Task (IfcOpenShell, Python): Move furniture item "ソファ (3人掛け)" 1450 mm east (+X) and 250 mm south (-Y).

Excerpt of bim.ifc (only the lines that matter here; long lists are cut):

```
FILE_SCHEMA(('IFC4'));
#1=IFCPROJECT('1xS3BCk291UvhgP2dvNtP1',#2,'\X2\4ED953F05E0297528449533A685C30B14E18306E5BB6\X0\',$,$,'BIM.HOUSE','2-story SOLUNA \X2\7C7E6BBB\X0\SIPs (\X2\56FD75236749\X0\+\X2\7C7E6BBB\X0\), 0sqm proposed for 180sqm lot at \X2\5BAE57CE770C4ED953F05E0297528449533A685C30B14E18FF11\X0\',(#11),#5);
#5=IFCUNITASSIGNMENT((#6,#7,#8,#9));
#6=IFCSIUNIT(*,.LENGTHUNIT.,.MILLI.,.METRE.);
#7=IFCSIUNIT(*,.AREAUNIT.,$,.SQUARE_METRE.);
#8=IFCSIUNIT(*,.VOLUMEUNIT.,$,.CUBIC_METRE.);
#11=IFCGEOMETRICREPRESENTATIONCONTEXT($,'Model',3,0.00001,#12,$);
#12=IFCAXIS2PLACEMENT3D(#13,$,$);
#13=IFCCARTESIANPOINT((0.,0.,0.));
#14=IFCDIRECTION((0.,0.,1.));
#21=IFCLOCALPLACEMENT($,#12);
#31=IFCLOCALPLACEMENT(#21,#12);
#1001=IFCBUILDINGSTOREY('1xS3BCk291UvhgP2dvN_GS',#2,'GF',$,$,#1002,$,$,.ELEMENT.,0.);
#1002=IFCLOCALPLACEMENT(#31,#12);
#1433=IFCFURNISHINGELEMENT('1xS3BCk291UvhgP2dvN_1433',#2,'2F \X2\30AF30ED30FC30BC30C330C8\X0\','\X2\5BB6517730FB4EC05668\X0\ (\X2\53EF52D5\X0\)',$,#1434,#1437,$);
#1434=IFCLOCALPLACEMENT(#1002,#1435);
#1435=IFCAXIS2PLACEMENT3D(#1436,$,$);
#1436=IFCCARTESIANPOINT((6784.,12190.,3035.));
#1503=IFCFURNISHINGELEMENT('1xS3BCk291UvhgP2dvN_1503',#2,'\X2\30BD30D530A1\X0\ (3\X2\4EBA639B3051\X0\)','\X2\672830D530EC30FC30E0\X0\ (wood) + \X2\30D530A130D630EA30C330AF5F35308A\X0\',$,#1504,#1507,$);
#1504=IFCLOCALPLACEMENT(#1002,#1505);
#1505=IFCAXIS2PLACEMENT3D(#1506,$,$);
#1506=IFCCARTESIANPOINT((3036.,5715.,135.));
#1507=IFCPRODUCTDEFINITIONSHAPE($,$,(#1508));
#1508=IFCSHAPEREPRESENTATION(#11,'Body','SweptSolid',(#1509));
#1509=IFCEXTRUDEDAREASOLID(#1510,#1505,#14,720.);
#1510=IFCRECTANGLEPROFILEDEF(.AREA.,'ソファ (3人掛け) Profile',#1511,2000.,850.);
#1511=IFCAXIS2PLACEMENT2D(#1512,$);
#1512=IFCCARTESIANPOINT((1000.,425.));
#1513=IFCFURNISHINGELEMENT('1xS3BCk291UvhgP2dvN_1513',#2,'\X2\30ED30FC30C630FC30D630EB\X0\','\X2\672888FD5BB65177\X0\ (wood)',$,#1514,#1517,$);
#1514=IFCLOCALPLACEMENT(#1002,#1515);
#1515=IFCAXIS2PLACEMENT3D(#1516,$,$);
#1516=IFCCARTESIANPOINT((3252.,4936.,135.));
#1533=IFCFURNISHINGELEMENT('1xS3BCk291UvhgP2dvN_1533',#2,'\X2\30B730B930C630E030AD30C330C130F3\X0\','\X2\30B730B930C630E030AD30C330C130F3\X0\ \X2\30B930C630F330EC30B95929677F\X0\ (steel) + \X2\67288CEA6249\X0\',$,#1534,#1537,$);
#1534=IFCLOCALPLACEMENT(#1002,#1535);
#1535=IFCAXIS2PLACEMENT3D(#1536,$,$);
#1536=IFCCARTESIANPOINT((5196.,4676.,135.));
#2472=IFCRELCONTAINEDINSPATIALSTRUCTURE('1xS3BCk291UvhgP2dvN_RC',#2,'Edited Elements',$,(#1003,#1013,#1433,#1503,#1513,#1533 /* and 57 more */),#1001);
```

```python
import ifcopenshell
import ifcopenshell.api.geometry
import ifcopenshell.util.placement

model = ifcopenshell.open("bim.ifc")

item = model.by_guid("1xS3BCk291UvhgP2dvN_1503")
matrix = ifcopenshell.util.placement.get_local_placement(item.ObjectPlacement)
matrix[0, 3] += 1450.0
matrix[1, 3] -= 250.0
ifcopenshell.api.geometry.edit_object_placement(model, product=item, matrix=matrix, is_si=False)

print(ifcopenshell.util.placement.get_local_placement(item.ObjectPlacement).round(3) + 0.0)

model.write("bim_v2.ifc")
```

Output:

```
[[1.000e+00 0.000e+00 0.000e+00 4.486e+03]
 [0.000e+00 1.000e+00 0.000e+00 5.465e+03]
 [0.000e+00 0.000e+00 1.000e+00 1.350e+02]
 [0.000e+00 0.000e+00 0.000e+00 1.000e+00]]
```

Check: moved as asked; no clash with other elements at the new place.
